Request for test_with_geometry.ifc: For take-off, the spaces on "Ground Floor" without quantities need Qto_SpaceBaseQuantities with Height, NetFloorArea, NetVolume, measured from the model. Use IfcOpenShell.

First a look at what the model holds.

```python
import ifcopenshell
import ifcopenshell.util.element
import ifcopenshell.util.unit

model = ifcopenshell.open("test_with_geometry.ifc")
print(model.schema)
for unit_type in ("LENGTHUNIT", "AREAUNIT", "VOLUMEUNIT"):
    print(unit_type, ifcopenshell.util.unit.calculate_unit_scale(model, unit_type))
storey = next(s for s in model.by_type("IfcBuildingStorey") if s.Name == "Ground Floor")
spaces = [e for e in ifcopenshell.util.element.get_decomposition(storey) if e.is_a("IfcSpace")]
for e in sorted(spaces, key=lambda e: e.id()):
    print(e.id(), e.is_a(), e.Name, list(ifcopenshell.util.element.get_psets(e, qtos_only=True)), sep=" | ")
```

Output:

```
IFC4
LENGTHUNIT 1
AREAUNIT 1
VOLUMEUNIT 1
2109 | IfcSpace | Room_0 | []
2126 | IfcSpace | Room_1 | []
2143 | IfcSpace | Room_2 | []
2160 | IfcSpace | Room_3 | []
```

```python
import ifcopenshell
import ifcopenshell.api.pset
import ifcopenshell.geom
import ifcopenshell.util.element
import ifcopenshell.util.shape
import ifcopenshell.util.unit

model = ifcopenshell.open("test_with_geometry.ifc")
unit_scale = ifcopenshell.util.unit.calculate_unit_scale(model)
area_scale = ifcopenshell.util.unit.calculate_unit_scale(model, "AREAUNIT")
volume_scale = ifcopenshell.util.unit.calculate_unit_scale(model, "VOLUMEUNIT")
settings = ifcopenshell.geom.settings()

storey = next(s for s in model.by_type("IfcBuildingStorey") if s.Name == "Ground Floor")
spaces = [e for e in ifcopenshell.util.element.get_decomposition(storey) if e.is_a("IfcSpace")]

for e in sorted(spaces, key=lambda e: e.id()):
    if ifcopenshell.util.element.get_psets(e, qtos_only=True, should_inherit=False):
        continue
    # Geometry comes back in metres, in the element's own axes.
    shape = ifcopenshell.geom.create_shape(settings, e)
    values = {
        "Height": ifcopenshell.util.shape.get_z(shape.geometry) / unit_scale,
        "NetFloorArea": ifcopenshell.util.shape.get_footprint_area(shape.geometry) / area_scale,
        "NetVolume": ifcopenshell.util.shape.get_volume(shape.geometry) / volume_scale,
    }
    qto = ifcopenshell.api.pset.add_qto(model, product=e, name="Qto_SpaceBaseQuantities")
    ifcopenshell.api.pset.edit_qto(model, qto=qto, properties=values)
    print(e.id(), {k: round(v, 3) for k, v in values.items()})

model.write("test_with_geometry_updated.ifc")
```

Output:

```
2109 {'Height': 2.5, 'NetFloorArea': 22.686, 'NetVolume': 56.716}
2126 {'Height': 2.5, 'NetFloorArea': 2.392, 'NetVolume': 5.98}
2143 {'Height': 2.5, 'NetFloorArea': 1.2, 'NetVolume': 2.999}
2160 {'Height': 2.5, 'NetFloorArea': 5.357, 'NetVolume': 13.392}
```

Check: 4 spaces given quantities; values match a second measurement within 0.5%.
